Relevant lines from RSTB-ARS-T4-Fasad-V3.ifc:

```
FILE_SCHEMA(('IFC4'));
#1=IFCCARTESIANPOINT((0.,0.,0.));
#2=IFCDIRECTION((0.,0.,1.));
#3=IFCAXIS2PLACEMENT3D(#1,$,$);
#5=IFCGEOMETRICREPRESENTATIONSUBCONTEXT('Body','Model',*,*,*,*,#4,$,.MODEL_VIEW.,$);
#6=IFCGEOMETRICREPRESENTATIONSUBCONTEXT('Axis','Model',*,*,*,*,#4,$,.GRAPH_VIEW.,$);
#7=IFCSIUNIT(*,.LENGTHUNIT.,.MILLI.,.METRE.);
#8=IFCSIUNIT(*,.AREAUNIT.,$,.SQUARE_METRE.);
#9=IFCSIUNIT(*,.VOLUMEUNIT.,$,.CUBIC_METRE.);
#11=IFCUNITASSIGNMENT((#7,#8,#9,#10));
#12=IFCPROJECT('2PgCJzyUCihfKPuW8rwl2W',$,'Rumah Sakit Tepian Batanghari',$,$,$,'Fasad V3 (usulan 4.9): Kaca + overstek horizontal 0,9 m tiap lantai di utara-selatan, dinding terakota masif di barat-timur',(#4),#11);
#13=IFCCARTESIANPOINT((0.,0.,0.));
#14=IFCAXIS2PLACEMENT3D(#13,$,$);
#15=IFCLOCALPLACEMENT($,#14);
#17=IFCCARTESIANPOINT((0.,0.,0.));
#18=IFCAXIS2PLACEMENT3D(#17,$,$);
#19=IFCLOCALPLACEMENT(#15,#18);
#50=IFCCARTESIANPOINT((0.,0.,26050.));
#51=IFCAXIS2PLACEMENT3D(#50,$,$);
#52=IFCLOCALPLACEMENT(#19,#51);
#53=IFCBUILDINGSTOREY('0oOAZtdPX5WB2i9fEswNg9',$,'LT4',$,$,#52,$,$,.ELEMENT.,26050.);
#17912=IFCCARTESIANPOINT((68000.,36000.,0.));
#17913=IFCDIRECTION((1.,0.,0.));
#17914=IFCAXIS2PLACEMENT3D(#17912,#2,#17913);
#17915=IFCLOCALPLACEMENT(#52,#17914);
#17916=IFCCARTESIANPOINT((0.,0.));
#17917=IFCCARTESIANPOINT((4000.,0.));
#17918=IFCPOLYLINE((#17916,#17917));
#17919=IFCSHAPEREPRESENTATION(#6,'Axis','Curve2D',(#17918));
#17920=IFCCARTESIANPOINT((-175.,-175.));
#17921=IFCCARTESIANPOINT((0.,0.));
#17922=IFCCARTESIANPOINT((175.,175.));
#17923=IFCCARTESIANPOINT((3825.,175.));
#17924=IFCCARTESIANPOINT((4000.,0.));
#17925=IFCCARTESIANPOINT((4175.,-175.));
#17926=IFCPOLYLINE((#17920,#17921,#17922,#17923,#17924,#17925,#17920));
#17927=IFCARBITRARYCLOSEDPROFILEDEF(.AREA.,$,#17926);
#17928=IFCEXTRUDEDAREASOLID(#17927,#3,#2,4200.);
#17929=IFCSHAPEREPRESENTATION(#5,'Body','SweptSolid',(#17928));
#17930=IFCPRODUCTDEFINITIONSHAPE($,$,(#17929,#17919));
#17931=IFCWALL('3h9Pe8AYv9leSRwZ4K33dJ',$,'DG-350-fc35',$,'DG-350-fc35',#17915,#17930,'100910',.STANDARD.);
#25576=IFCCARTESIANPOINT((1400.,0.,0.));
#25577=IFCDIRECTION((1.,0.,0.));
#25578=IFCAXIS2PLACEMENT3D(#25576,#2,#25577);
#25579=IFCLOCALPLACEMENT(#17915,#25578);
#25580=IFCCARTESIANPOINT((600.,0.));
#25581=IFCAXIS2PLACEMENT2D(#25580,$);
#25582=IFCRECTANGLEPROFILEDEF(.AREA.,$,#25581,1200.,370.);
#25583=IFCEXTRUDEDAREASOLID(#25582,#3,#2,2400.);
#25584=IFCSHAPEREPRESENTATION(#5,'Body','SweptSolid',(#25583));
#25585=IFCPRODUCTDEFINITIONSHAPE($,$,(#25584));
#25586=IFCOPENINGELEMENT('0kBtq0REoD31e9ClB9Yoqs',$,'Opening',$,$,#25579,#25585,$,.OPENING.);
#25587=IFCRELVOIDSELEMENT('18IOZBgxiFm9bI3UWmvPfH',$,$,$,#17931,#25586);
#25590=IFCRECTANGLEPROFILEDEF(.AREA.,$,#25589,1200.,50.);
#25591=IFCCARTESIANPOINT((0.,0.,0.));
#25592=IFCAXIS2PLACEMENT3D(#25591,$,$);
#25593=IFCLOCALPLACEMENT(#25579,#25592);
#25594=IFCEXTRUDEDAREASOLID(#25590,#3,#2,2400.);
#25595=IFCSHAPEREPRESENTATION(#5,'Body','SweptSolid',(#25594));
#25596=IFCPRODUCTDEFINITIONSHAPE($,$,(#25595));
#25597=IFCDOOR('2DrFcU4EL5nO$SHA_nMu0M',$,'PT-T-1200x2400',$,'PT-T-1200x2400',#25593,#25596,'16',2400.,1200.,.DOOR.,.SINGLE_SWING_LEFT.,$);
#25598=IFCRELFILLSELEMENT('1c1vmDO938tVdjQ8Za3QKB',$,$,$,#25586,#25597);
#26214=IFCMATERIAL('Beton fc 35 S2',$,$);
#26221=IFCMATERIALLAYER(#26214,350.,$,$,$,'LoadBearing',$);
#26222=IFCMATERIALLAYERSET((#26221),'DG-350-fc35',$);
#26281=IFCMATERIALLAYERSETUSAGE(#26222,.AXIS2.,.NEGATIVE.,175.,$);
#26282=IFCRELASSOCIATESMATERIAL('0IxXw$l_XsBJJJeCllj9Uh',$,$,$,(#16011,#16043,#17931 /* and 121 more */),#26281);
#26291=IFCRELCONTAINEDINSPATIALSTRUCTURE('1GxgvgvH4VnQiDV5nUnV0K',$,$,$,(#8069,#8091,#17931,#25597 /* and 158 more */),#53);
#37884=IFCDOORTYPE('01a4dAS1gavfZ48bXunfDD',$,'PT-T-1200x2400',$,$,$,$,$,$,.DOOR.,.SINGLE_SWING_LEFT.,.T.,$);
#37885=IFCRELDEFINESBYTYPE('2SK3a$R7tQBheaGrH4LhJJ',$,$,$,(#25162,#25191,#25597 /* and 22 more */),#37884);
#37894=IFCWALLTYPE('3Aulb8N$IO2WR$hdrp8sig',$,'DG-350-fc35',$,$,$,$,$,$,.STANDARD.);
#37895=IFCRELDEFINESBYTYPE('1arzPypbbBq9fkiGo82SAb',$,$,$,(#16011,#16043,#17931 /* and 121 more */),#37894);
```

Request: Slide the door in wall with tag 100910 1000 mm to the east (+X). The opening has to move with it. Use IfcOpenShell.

```python
import ifcopenshell
import ifcopenshell.api.geometry
import ifcopenshell.util.placement
import ifcopenshell.util.unit

model = ifcopenshell.open("RSTB-ARS-T4-Fasad-V3.ifc")
unit_scale = ifcopenshell.util.unit.calculate_unit_scale(model)

door = model.by_guid("2DrFcU4EL5nO$SHA_nMu0M")
opening = door.FillsVoids[0].RelatingOpeningElement
wall = opening.VoidsElements[0].RelatingBuildingElement

wall_matrix = ifcopenshell.util.placement.get_local_placement(wall.ObjectPlacement)
shift = wall_matrix[:3, 0] * 1 / unit_scale
before = ifcopenshell.util.placement.get_local_placement(door.ObjectPlacement)[:3, 3].copy()

# The door is placed relative to its opening, so it follows when the opening moves.
matrix = ifcopenshell.util.placement.get_local_placement(opening.ObjectPlacement)
matrix[:3, 3] += shift
ifcopenshell.api.geometry.edit_object_placement(
    model, product=opening, matrix=matrix, is_si=False, should_transform_children=True
)

after = ifcopenshell.util.placement.get_local_placement(door.ObjectPlacement)[:3, 3]
print("door moved by", (after - before).round(3) + 0.0)

model.write("RSTB-ARS-T4-Fasad-V3_edited.ifc")
```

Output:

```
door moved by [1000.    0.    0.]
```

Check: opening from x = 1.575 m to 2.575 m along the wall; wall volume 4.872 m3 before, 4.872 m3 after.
